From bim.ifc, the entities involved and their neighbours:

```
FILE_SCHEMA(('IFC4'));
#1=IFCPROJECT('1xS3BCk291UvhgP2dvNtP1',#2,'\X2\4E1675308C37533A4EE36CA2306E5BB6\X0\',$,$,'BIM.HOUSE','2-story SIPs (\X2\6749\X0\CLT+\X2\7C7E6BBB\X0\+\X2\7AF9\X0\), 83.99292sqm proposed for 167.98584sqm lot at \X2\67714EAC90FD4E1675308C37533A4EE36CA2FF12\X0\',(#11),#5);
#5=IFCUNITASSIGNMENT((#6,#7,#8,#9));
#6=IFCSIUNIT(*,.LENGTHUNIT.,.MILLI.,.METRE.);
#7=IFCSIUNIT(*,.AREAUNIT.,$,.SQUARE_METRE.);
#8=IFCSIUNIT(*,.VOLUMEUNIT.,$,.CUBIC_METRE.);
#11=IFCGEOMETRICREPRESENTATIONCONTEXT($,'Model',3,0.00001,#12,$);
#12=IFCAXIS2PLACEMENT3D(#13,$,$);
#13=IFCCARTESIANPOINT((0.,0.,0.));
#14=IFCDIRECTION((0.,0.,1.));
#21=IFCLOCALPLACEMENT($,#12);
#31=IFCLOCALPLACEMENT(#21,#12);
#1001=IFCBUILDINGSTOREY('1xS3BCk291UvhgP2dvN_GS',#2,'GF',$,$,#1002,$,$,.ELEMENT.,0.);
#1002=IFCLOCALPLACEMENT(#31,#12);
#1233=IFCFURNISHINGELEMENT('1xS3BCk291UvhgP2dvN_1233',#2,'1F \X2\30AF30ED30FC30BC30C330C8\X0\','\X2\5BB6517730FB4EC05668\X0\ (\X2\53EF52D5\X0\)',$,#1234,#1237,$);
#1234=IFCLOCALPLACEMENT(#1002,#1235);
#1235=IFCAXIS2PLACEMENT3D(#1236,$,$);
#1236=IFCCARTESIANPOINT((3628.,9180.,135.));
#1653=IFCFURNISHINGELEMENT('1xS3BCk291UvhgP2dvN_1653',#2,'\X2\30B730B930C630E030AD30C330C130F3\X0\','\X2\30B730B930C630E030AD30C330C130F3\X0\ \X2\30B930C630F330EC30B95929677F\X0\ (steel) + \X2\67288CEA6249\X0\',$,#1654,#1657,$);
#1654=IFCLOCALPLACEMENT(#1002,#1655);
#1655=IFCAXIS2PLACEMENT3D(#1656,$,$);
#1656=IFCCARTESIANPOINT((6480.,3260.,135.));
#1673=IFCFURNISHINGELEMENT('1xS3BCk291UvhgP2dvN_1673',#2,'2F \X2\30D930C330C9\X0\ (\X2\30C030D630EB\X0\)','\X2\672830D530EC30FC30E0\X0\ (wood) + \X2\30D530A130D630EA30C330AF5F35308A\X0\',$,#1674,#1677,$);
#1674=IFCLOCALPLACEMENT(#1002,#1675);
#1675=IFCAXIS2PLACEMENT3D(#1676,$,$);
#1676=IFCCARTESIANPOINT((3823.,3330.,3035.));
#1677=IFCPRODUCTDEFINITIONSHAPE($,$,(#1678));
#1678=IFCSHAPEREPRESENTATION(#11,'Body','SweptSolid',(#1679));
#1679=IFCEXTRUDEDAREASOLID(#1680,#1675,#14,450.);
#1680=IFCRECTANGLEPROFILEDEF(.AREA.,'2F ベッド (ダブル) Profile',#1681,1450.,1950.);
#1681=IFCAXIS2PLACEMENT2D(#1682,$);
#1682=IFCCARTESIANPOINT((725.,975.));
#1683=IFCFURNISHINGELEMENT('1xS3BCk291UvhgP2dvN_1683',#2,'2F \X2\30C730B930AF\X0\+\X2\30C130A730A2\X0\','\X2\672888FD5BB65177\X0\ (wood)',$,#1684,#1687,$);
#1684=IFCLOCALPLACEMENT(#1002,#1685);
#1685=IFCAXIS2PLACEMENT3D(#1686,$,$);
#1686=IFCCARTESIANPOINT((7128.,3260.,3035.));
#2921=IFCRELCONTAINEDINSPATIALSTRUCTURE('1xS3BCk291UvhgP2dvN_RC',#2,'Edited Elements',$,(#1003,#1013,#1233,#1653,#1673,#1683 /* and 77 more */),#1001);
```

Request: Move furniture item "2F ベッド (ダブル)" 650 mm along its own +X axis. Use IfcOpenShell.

```python
import ifcopenshell
import ifcopenshell.api.geometry
import ifcopenshell.util.placement
import ifcopenshell.util.unit

model = ifcopenshell.open("bim.ifc")
unit_scale = ifcopenshell.util.unit.calculate_unit_scale(model)

item = model.by_guid("1xS3BCk291UvhgP2dvN_1673")
matrix = ifcopenshell.util.placement.get_local_placement(item.ObjectPlacement)
matrix[:3, 3] += matrix[:3, 0] * 0.65 / unit_scale
ifcopenshell.api.geometry.edit_object_placement(model, product=item, matrix=matrix, is_si=False)

print(ifcopenshell.util.placement.get_local_placement(item.ObjectPlacement).round(3) + 0.0)

model.write("bim_rev.ifc")
```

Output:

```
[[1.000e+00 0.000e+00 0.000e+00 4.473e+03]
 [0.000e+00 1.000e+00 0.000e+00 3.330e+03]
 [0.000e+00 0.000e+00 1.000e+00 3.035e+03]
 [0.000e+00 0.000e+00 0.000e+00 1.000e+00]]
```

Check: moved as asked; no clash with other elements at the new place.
